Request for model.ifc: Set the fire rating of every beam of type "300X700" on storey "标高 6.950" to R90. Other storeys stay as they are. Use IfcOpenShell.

First a look at what the model holds.

```python
import ifcopenshell
import ifcopenshell.util.element

model = ifcopenshell.open("model.ifc")
print(model.schema)
storey = next(s for s in model.by_type("IfcBuildingStorey") if s.Name == "标高 6.950")
beams = [e for e in ifcopenshell.util.element.get_decomposition(storey) if e.is_a("IfcBeam")]
seen = {}
for e in beams:
    element_type = ifcopenshell.util.element.get_type(e)
    key = (element_type.Name if element_type != e and element_type else None, ifcopenshell.util.element.get_pset(e, "Pset_BeamCommon", "FireRating"))
    seen[key] = seen.get(key, 0) + 1
for (name, value), count in sorted(seen.items(), key=str):
    print(count, "x", name, "|", value)
```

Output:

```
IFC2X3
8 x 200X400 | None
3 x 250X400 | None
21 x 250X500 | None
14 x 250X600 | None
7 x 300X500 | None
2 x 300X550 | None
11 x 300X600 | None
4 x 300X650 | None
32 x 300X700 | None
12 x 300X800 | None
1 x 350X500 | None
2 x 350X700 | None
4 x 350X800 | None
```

```python
import ifcopenshell
import ifcopenshell.api.pset
import ifcopenshell.util.element

model = ifcopenshell.open("model.ifc")

storey = next(s for s in model.by_type("IfcBuildingStorey") if s.Name == "标高 6.950")
beams = [e for e in ifcopenshell.util.element.get_decomposition(storey) if e.is_a("IfcBeam")]

count = 0
for e in beams:
    element_type = ifcopenshell.util.element.get_type(e)
    if element_type in (None, e) or element_type.Name != "300X700":
        continue
    # add_pset returns the element's existing set when there is one.
    pset = ifcopenshell.api.pset.add_pset(model, product=e, name="Pset_BeamCommon")
    ifcopenshell.api.pset.edit_pset(model, pset=pset, properties={"FireRating": "R90"})
    count += 1

print(count, "beams updated")

model.write("model_v2.ifc")
```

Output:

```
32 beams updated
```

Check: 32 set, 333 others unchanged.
